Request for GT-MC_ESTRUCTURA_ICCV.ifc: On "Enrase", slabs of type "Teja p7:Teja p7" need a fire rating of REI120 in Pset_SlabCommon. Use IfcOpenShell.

First a look at what the model holds.

```python
import ifcopenshell
import ifcopenshell.util.element

model = ifcopenshell.open("GT-MC_ESTRUCTURA_ICCV.ifc")
print(model.schema)
storey = next(s for s in model.by_type("IfcBuildingStorey") if s.Name == "Enrase")
slabs = [e for e in ifcopenshell.util.element.get_decomposition(storey) if e.is_a("IfcSlab")]
seen = {}
for e in slabs:
    element_type = ifcopenshell.util.element.get_type(e)
    key = (element_type.Name if element_type != e and element_type else None, ifcopenshell.util.element.get_pset(e, "Pset_SlabCommon", "FireRating"))
    seen[key] = seen.get(key, 0) + 1
for (name, value), count in sorted(seen.items(), key=str):
    print(count, "x", name, "|", value)
```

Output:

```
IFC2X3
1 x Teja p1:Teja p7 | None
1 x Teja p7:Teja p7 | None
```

```python
import ifcopenshell
import ifcopenshell.api.pset
import ifcopenshell.util.element

model = ifcopenshell.open("GT-MC_ESTRUCTURA_ICCV.ifc")

storey = next(s for s in model.by_type("IfcBuildingStorey") if s.Name == "Enrase")
slabs = [e for e in ifcopenshell.util.element.get_decomposition(storey) if e.is_a("IfcSlab")]

count = 0
for e in slabs:
    element_type = ifcopenshell.util.element.get_type(e)
    if element_type in (None, e) or element_type.Name != "Teja p7:Teja p7":
        continue
    # add_pset returns the element's existing set when there is one.
    pset = ifcopenshell.api.pset.add_pset(model, product=e, name="Pset_SlabCommon")
    ifcopenshell.api.pset.edit_pset(model, pset=pset, properties={"FireRating": "REI120"})
    count += 1

print(count, "slabs updated")

model.write("GT-MC_ESTRUCTURA_ICCV_rev.ifc")
```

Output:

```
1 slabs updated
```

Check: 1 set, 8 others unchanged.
